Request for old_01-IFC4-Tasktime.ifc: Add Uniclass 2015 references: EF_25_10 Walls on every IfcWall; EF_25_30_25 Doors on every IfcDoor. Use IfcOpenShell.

First a look at what the model holds.

```python
import ifcopenshell

model = ifcopenshell.open("old_01-IFC4-Tasktime.ifc")
print(model.schema)
print("classifications:", [c.Name for c in model.by_type("IfcClassification")])
for ifc_class in ("IfcDoor", "IfcRoof", "IfcStair", "IfcWall", "IfcWindow"):
    print(ifc_class, len(model.by_type(ifc_class)))
```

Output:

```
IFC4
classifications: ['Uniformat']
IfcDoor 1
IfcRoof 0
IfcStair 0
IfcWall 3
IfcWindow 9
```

```python
import ifcopenshell
import ifcopenshell.api.classification

model = ifcopenshell.open("old_01-IFC4-Tasktime.ifc")

system = ifcopenshell.api.classification.add_classification(model, classification="Uniclass 2015")

codes = {
    "IfcWall": ("EF_25_10", "Walls"),
    "IfcDoor": ("EF_25_30_25", "Doors"),
}
for ifc_class, (code, name) in codes.items():
    products = model.by_type(ifc_class)
    ifcopenshell.api.classification.add_reference(
        model, products=products, classification=system, identification=code, name=name
    )
    print(code, len(products))

model.write("old_01-IFC4-Tasktime_edited.ifc")
```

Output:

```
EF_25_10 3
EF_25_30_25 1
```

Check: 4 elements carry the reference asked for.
